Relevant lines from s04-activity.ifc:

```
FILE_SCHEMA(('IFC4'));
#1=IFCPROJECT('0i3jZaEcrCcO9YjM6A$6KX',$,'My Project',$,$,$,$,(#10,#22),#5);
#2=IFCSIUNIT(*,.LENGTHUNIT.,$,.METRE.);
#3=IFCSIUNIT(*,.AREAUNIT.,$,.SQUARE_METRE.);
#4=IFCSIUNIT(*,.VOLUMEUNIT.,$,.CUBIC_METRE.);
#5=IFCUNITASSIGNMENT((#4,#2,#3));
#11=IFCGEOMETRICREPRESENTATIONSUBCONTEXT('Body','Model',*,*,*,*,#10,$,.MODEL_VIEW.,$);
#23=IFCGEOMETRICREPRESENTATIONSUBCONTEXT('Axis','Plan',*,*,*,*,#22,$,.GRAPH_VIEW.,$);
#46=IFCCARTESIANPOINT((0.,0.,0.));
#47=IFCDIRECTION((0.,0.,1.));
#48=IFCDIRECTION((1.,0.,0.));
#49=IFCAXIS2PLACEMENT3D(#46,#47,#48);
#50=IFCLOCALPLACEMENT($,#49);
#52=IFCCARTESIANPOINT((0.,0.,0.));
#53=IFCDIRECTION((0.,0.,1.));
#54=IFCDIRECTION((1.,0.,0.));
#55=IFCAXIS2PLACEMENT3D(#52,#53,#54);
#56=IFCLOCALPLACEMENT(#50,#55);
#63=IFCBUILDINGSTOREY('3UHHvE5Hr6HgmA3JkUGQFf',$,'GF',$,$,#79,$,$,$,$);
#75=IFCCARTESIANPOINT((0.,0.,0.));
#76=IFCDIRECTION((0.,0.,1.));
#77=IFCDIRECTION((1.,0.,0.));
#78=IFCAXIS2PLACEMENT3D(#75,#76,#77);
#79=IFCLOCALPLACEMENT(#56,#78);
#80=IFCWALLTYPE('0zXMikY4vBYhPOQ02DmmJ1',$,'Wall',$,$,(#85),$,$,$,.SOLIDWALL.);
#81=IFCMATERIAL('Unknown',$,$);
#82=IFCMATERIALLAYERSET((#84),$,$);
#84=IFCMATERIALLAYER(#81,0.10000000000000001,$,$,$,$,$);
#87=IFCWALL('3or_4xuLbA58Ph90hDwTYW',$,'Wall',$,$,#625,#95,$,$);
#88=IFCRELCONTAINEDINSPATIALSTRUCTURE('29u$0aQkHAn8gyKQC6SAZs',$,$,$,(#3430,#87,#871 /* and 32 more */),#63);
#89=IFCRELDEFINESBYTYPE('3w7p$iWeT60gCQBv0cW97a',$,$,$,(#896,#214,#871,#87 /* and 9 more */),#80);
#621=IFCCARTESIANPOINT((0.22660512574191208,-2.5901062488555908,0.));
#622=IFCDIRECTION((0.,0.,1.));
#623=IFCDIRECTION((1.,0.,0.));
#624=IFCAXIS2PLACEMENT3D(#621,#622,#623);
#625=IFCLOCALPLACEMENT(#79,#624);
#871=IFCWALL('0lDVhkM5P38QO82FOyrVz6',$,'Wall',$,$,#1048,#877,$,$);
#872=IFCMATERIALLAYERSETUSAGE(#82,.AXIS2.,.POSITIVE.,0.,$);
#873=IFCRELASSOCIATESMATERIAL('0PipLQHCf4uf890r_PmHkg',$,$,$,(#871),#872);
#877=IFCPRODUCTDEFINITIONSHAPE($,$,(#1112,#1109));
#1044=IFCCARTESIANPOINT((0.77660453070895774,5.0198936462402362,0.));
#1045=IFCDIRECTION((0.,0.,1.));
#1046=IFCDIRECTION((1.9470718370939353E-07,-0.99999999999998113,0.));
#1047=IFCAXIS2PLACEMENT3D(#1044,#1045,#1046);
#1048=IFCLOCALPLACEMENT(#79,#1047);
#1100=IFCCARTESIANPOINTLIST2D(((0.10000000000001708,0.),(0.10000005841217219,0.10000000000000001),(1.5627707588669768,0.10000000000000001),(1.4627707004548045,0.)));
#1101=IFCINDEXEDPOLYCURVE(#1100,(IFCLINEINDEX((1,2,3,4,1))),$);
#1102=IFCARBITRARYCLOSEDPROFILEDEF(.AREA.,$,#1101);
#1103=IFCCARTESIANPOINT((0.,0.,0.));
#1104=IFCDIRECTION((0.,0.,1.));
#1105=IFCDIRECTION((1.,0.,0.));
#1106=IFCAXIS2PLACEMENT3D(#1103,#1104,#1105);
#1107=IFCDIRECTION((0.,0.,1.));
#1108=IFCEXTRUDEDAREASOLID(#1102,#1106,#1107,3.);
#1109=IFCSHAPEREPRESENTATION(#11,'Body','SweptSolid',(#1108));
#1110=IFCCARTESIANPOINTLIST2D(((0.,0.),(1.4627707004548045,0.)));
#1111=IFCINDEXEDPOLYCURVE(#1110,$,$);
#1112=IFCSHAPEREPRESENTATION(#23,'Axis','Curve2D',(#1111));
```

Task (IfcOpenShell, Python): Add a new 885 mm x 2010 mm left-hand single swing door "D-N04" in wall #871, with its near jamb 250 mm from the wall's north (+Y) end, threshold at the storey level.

```python
import numpy as np
import ifcopenshell
import ifcopenshell.api.feature
import ifcopenshell.api.geometry
import ifcopenshell.api.root
import ifcopenshell.api.spatial
import ifcopenshell.geom
import ifcopenshell.util.element
import ifcopenshell.util.placement
import ifcopenshell.util.representation
import ifcopenshell.util.shape
import ifcopenshell.util.unit

model = ifcopenshell.open("s04-activity.ifc")
unit_scale = ifcopenshell.util.unit.calculate_unit_scale(model)
settings = ifcopenshell.geom.settings()


def volume(element):
    """Net volume in cubic metres, openings subtracted."""
    shape = ifcopenshell.geom.create_shape(settings, element)
    return ifcopenshell.util.shape.get_volume(shape.geometry)


wall = model.by_guid("0lDVhkM5P38QO82FOyrVz6")
storey = ifcopenshell.util.element.get_container(wall, ifc_class="IfcBuildingStorey")
context = ifcopenshell.util.representation.get_context(model, "Model", "Body", "MODEL_VIEW")
before = volume(wall)

width, height, from_end, sill = 0.885, 2.01, 0.25, 0.0  # metres

# The wall runs along its own X axis, and the end named is its -X end.
wall_shape = ifcopenshell.geom.create_shape(settings, wall)
x, y, z = ifcopenshell.util.shape.get_vertices(wall_shape.geometry).T
start = x.min() + from_end
face, thickness = float(y.min()), float(y.max() - y.min())
wall_matrix = ifcopenshell.util.placement.get_local_placement(wall.ObjectPlacement)
level = ifcopenshell.util.placement.get_local_placement(storey.ObjectPlacement)[2, 3]


def in_wall(x, y):
    """Placement at x, y metres in the wall's axes, at sill height."""
    matrix = wall_matrix.copy()
    matrix[:, 3] = wall_matrix @ np.array([x / unit_scale, y / unit_scale, 0.0, 1.0])
    matrix[2, 3] = level + sill / unit_scale
    return matrix


# Opening: a box that overshoots both wall faces by 50 mm.
opening = ifcopenshell.api.root.create_entity(model, ifc_class="IfcOpeningElement", predefined_type="OPENING")
box = ifcopenshell.api.geometry.add_wall_representation(
    model, context=context, length=width, height=height, thickness=thickness + 0.1
)
ifcopenshell.api.geometry.assign_representation(model, product=opening, representation=box)
ifcopenshell.api.geometry.edit_object_placement(model, product=opening, matrix=in_wall(start, face - 0.05), is_si=False)
ifcopenshell.api.feature.add_feature(model, feature=opening, element=wall)

door = ifcopenshell.api.root.create_entity(model, ifc_class="IfcDoor", name="D-N04", predefined_type="DOOR")
door.OverallWidth, door.OverallHeight = width / unit_scale, height / unit_scale
door.OperationType = "SINGLE_SWING_LEFT"
body = ifcopenshell.api.geometry.add_door_representation(
    model,
    context=context,
    overall_width=door.OverallWidth,
    overall_height=door.OverallHeight,
    operation_type="SINGLE_SWING_LEFT",
    lining_properties={"LiningDepth": thickness / unit_scale, "ThresholdDepth": thickness / unit_scale},
)
ifcopenshell.api.geometry.assign_representation(model, product=door, representation=body)
ifcopenshell.api.spatial.assign_container(model, products=[door], relating_structure=storey)
ifcopenshell.api.feature.add_filling(model, opening=opening, element=door)

# The lining spans the wall, so the door starts at the wall face.
ifcopenshell.api.geometry.edit_object_placement(model, product=door, matrix=in_wall(start, face), is_si=False)

after = volume(wall)

print(f"wall volume {before:.3f} -> {after:.3f} m3")

model.write("s04-activity_v2.ifc")
```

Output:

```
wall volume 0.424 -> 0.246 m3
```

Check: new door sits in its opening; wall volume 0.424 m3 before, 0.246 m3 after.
